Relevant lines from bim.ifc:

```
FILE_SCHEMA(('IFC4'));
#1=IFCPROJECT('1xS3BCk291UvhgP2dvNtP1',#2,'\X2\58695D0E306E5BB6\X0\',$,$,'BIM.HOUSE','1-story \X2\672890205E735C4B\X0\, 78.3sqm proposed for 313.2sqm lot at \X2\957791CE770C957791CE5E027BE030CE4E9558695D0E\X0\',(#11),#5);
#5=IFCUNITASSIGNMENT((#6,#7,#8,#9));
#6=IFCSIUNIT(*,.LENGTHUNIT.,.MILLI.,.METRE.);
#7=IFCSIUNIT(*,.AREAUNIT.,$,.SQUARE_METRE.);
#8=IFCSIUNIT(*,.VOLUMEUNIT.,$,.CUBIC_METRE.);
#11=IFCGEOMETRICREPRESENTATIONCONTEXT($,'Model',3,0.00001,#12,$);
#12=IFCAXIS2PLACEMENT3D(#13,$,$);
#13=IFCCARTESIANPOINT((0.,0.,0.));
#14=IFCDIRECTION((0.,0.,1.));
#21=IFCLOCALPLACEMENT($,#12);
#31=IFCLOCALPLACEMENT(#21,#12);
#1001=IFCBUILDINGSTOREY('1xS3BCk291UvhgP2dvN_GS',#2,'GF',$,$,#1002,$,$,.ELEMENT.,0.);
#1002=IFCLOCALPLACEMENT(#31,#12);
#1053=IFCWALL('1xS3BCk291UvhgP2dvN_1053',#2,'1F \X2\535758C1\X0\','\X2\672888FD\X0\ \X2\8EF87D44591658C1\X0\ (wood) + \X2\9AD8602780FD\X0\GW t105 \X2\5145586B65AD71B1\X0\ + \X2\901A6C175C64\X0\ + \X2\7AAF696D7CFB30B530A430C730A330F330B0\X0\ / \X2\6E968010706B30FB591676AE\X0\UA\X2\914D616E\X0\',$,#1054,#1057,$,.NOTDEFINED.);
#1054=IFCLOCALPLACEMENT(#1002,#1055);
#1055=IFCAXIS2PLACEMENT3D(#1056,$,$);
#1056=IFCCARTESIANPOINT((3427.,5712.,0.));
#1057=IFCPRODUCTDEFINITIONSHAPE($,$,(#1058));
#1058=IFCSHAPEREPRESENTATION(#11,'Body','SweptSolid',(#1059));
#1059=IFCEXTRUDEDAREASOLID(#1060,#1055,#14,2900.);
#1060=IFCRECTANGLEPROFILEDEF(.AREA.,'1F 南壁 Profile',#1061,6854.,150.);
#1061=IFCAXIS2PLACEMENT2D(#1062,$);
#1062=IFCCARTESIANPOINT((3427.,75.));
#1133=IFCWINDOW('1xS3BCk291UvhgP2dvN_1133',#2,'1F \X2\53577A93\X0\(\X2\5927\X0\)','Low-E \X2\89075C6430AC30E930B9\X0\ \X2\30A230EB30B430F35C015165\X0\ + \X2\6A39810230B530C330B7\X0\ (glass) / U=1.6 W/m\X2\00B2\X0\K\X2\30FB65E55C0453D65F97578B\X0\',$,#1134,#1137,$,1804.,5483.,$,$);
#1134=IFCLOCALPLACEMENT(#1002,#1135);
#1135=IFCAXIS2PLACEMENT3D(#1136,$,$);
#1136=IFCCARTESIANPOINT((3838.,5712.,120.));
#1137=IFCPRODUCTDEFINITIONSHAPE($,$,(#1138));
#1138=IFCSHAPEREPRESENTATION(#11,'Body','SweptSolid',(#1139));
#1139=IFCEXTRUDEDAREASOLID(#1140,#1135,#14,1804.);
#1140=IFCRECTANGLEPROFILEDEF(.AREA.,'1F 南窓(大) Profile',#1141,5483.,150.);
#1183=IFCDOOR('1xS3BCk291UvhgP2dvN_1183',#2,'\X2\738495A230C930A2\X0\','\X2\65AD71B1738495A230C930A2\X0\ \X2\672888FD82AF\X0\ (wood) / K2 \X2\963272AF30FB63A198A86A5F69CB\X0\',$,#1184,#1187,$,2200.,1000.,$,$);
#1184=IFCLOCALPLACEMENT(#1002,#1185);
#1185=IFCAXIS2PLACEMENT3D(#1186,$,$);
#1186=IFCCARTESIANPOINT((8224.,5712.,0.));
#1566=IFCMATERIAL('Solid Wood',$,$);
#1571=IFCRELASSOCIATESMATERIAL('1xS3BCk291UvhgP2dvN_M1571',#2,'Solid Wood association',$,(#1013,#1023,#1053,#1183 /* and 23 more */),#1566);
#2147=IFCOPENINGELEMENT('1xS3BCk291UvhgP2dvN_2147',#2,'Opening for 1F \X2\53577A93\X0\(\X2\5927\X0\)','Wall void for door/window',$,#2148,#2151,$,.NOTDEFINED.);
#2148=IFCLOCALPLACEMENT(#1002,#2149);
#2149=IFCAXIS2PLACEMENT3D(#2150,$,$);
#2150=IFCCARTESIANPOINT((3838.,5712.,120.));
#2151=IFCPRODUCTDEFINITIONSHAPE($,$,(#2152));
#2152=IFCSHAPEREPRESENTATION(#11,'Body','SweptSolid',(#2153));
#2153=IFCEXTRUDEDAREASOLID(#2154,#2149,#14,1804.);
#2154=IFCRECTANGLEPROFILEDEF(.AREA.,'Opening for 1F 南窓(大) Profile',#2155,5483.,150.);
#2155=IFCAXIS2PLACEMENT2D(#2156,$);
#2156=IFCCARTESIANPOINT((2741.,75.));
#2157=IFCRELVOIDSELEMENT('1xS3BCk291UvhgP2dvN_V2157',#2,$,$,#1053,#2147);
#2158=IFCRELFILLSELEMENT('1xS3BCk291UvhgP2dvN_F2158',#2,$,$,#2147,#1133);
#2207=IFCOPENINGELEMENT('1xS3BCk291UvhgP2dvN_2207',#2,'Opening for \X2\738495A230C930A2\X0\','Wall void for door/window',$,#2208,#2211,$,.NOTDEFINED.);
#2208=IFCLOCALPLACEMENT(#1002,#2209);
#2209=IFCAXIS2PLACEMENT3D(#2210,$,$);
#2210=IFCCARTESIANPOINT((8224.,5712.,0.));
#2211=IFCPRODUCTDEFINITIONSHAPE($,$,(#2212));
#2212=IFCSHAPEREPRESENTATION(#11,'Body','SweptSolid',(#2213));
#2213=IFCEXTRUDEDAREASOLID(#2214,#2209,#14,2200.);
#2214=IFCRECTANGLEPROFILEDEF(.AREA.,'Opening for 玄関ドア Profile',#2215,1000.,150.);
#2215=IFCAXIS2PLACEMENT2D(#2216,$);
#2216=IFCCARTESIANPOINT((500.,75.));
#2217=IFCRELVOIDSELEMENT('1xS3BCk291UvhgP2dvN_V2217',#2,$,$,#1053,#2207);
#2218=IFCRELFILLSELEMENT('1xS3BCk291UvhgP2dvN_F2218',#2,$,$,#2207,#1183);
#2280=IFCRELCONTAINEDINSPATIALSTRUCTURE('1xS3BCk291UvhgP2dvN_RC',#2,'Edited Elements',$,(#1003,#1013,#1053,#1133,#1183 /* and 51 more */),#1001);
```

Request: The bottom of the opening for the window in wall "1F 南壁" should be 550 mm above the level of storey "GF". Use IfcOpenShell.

```python
import numpy as np
import ifcopenshell
import ifcopenshell.api.geometry
import ifcopenshell.geom
import ifcopenshell.util.element
import ifcopenshell.util.placement
import ifcopenshell.util.shape
import ifcopenshell.util.unit

model = ifcopenshell.open("bim.ifc")
unit_scale = ifcopenshell.util.unit.calculate_unit_scale(model)

window = model.by_guid("1xS3BCk291UvhgP2dvN_1133")
opening = window.FillsVoids[0].RelatingOpeningElement
storey = ifcopenshell.util.element.get_container(window, ifc_class="IfcBuildingStorey")
level = ifcopenshell.util.placement.get_local_placement(storey.ObjectPlacement)[2, 3]

# The opening's origin need not be at the sill, so measure its lowest point.
shape = ifcopenshell.geom.create_shape(ifcopenshell.geom.settings(), opening)
bottom = ifcopenshell.util.shape.get_shape_bottom_elevation(shape, shape.geometry) / unit_scale
dz = level + 0.55 / unit_scale - bottom

shift = np.array([0.0, 0.0, dz])
# The window is not placed relative to its opening, so move both.
for product in (opening, window):
    matrix = ifcopenshell.util.placement.get_local_placement(product.ObjectPlacement)
    matrix[:3, 3] += shift
    ifcopenshell.api.geometry.edit_object_placement(model, product=product, matrix=matrix, is_si=False)

print(f"moved by {dz * unit_scale:+.3f} m")

model.write("bim_rev.ifc")
```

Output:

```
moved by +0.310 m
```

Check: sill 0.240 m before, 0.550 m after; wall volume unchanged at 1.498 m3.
